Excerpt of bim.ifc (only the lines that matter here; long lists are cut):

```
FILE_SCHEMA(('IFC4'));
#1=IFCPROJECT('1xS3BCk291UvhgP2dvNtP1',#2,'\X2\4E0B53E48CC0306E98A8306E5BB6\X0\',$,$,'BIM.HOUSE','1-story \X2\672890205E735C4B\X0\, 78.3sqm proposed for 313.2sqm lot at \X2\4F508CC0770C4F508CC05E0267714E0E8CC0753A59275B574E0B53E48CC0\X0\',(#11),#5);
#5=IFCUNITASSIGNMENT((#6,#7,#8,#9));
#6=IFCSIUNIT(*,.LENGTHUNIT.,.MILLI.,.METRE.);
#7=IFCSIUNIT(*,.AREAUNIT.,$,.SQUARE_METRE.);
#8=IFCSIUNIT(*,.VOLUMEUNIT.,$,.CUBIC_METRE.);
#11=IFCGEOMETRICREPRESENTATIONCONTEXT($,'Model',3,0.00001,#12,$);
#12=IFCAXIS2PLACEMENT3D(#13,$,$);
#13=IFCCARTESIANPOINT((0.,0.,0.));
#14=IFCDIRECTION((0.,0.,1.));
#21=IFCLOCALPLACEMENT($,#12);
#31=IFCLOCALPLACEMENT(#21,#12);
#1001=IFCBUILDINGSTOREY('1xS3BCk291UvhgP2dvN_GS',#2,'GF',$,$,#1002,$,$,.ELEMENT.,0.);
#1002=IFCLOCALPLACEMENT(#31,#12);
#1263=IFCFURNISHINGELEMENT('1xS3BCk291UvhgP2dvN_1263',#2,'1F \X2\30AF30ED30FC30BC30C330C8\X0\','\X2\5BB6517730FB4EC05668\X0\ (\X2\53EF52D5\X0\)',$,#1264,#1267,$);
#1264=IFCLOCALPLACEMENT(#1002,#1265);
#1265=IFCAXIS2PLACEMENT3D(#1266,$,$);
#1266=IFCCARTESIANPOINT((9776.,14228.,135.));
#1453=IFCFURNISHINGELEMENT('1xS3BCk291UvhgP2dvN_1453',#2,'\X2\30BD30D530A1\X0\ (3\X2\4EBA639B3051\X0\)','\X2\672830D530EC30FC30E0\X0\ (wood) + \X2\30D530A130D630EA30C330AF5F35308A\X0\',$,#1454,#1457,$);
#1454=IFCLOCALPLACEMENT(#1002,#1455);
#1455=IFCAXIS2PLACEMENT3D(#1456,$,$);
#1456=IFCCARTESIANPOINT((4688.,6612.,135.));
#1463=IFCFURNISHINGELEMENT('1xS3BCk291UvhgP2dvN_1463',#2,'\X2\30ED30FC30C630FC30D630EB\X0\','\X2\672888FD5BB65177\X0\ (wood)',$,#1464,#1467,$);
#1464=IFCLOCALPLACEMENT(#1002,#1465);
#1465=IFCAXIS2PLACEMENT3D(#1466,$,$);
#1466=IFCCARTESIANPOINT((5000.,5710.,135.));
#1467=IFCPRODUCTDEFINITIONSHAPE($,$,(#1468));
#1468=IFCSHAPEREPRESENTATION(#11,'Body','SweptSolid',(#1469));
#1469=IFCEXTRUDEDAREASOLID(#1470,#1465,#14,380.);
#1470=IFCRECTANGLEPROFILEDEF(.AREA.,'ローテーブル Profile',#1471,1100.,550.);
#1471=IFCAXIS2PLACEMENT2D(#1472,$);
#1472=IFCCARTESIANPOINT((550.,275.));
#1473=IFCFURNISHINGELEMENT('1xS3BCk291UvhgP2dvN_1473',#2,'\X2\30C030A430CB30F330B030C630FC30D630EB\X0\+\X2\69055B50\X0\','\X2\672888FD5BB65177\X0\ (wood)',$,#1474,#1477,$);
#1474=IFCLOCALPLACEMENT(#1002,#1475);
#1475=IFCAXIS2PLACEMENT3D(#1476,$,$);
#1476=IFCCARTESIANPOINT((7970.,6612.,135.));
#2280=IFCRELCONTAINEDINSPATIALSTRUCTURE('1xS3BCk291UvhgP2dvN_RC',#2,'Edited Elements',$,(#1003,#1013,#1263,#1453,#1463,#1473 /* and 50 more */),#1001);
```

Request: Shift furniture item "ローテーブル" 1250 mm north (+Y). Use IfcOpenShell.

```python
import ifcopenshell
import ifcopenshell.api.geometry
import ifcopenshell.util.placement

model = ifcopenshell.open("bim.ifc")

item = model.by_guid("1xS3BCk291UvhgP2dvN_1463")
matrix = ifcopenshell.util.placement.get_local_placement(item.ObjectPlacement)
matrix[1, 3] += 1250.0
ifcopenshell.api.geometry.edit_object_placement(model, product=item, matrix=matrix, is_si=False)

print(ifcopenshell.util.placement.get_local_placement(item.ObjectPlacement).round(3) + 0.0)

model.write("bim_rev.ifc")
```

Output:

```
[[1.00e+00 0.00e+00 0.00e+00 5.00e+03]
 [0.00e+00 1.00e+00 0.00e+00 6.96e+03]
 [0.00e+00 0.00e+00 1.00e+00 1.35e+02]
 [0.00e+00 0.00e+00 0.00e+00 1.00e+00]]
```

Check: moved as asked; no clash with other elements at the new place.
